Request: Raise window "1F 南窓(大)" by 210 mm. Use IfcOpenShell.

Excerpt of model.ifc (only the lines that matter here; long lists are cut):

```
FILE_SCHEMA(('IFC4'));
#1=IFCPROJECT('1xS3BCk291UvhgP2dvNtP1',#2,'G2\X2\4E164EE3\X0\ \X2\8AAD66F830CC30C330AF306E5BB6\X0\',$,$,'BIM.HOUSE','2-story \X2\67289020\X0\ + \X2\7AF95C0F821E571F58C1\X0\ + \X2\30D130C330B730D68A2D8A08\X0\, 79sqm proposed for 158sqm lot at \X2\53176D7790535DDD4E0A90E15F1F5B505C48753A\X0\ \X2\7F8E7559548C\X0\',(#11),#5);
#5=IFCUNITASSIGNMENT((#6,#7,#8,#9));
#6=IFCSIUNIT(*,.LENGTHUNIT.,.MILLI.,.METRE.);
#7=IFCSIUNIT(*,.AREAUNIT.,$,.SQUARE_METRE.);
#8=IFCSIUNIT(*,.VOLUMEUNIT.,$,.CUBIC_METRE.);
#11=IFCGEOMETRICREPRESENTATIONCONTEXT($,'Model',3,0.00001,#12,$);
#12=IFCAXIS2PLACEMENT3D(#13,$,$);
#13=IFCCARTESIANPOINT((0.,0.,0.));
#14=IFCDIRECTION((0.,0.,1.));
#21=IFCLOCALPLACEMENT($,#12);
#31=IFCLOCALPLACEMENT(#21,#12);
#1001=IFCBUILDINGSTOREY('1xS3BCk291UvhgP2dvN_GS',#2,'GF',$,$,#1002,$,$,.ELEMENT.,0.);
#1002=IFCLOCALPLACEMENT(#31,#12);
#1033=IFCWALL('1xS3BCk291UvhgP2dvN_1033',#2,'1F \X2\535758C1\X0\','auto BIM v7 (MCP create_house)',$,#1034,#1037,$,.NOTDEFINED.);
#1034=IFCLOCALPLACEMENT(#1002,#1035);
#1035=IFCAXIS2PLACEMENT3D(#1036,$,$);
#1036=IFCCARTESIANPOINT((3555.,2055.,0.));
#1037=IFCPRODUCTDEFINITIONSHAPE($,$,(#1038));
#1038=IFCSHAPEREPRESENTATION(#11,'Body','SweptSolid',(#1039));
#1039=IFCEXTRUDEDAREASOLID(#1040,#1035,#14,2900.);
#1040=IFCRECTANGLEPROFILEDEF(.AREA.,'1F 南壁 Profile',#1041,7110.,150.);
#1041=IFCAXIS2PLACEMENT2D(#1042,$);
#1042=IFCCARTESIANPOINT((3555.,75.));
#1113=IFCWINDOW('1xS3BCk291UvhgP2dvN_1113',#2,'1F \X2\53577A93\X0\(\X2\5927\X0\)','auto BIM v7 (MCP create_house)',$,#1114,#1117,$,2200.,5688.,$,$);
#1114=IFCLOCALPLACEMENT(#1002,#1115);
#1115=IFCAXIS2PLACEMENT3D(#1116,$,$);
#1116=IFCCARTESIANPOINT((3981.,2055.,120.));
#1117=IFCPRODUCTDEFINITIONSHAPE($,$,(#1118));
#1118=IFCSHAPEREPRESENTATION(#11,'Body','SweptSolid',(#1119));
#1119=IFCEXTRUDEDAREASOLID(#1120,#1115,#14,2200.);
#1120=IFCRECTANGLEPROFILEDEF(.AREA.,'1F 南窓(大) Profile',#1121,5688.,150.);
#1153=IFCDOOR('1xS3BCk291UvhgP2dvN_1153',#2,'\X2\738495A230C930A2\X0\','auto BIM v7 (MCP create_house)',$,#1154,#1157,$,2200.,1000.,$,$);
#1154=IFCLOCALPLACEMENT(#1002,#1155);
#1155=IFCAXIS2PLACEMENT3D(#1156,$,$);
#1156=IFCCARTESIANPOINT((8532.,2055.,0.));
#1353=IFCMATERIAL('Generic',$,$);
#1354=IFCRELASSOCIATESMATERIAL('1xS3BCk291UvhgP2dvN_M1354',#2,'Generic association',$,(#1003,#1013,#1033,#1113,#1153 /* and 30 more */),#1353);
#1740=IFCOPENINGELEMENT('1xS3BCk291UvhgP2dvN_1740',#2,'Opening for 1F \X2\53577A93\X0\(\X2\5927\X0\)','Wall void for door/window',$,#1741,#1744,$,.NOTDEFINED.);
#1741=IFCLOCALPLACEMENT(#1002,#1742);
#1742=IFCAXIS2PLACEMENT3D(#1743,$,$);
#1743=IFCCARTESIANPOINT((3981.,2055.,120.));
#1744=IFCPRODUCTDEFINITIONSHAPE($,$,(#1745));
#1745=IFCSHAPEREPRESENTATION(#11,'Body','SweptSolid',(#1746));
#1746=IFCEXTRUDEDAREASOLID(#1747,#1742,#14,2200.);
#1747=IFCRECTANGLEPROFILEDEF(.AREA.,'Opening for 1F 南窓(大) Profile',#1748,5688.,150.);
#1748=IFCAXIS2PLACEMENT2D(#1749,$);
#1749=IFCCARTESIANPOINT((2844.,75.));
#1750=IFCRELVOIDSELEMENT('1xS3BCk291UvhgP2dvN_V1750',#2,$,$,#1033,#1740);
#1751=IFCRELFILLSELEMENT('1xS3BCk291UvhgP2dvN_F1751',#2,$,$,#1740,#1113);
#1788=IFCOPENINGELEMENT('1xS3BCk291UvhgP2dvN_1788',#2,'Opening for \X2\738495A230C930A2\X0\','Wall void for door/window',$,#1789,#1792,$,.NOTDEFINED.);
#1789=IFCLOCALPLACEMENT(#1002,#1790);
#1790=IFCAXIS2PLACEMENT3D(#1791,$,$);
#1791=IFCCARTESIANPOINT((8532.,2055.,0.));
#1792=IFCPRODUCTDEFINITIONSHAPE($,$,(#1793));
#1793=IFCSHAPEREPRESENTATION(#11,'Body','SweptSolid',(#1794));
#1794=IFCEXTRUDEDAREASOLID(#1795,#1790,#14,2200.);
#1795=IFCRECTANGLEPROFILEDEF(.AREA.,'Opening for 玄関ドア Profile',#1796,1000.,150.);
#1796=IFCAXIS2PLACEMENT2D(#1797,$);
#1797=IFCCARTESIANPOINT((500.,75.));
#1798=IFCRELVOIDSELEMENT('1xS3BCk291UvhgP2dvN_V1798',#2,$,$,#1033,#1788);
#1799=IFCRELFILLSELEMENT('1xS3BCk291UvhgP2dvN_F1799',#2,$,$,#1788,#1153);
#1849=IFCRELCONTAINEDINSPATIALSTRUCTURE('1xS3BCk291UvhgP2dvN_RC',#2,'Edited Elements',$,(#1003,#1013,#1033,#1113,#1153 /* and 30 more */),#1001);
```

```python
import numpy as np
import ifcopenshell
import ifcopenshell.api.geometry
import ifcopenshell.util.placement
import ifcopenshell.util.unit

model = ifcopenshell.open("model.ifc")
unit_scale = ifcopenshell.util.unit.calculate_unit_scale(model)

window = model.by_id(1113)
opening = window.FillsVoids[0].RelatingOpeningElement
dz = 0.21 / unit_scale

shift = np.array([0.0, 0.0, dz])
# The window is not placed relative to its opening, so move both.
for product in (opening, window):
    matrix = ifcopenshell.util.placement.get_local_placement(product.ObjectPlacement)
    matrix[:3, 3] += shift
    ifcopenshell.api.geometry.edit_object_placement(model, product=product, matrix=matrix, is_si=False)

print(f"moved by {dz * unit_scale:+.3f} m")

model.write("model_v2.ifc")
```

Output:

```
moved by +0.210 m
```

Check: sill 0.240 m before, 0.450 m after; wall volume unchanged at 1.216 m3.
